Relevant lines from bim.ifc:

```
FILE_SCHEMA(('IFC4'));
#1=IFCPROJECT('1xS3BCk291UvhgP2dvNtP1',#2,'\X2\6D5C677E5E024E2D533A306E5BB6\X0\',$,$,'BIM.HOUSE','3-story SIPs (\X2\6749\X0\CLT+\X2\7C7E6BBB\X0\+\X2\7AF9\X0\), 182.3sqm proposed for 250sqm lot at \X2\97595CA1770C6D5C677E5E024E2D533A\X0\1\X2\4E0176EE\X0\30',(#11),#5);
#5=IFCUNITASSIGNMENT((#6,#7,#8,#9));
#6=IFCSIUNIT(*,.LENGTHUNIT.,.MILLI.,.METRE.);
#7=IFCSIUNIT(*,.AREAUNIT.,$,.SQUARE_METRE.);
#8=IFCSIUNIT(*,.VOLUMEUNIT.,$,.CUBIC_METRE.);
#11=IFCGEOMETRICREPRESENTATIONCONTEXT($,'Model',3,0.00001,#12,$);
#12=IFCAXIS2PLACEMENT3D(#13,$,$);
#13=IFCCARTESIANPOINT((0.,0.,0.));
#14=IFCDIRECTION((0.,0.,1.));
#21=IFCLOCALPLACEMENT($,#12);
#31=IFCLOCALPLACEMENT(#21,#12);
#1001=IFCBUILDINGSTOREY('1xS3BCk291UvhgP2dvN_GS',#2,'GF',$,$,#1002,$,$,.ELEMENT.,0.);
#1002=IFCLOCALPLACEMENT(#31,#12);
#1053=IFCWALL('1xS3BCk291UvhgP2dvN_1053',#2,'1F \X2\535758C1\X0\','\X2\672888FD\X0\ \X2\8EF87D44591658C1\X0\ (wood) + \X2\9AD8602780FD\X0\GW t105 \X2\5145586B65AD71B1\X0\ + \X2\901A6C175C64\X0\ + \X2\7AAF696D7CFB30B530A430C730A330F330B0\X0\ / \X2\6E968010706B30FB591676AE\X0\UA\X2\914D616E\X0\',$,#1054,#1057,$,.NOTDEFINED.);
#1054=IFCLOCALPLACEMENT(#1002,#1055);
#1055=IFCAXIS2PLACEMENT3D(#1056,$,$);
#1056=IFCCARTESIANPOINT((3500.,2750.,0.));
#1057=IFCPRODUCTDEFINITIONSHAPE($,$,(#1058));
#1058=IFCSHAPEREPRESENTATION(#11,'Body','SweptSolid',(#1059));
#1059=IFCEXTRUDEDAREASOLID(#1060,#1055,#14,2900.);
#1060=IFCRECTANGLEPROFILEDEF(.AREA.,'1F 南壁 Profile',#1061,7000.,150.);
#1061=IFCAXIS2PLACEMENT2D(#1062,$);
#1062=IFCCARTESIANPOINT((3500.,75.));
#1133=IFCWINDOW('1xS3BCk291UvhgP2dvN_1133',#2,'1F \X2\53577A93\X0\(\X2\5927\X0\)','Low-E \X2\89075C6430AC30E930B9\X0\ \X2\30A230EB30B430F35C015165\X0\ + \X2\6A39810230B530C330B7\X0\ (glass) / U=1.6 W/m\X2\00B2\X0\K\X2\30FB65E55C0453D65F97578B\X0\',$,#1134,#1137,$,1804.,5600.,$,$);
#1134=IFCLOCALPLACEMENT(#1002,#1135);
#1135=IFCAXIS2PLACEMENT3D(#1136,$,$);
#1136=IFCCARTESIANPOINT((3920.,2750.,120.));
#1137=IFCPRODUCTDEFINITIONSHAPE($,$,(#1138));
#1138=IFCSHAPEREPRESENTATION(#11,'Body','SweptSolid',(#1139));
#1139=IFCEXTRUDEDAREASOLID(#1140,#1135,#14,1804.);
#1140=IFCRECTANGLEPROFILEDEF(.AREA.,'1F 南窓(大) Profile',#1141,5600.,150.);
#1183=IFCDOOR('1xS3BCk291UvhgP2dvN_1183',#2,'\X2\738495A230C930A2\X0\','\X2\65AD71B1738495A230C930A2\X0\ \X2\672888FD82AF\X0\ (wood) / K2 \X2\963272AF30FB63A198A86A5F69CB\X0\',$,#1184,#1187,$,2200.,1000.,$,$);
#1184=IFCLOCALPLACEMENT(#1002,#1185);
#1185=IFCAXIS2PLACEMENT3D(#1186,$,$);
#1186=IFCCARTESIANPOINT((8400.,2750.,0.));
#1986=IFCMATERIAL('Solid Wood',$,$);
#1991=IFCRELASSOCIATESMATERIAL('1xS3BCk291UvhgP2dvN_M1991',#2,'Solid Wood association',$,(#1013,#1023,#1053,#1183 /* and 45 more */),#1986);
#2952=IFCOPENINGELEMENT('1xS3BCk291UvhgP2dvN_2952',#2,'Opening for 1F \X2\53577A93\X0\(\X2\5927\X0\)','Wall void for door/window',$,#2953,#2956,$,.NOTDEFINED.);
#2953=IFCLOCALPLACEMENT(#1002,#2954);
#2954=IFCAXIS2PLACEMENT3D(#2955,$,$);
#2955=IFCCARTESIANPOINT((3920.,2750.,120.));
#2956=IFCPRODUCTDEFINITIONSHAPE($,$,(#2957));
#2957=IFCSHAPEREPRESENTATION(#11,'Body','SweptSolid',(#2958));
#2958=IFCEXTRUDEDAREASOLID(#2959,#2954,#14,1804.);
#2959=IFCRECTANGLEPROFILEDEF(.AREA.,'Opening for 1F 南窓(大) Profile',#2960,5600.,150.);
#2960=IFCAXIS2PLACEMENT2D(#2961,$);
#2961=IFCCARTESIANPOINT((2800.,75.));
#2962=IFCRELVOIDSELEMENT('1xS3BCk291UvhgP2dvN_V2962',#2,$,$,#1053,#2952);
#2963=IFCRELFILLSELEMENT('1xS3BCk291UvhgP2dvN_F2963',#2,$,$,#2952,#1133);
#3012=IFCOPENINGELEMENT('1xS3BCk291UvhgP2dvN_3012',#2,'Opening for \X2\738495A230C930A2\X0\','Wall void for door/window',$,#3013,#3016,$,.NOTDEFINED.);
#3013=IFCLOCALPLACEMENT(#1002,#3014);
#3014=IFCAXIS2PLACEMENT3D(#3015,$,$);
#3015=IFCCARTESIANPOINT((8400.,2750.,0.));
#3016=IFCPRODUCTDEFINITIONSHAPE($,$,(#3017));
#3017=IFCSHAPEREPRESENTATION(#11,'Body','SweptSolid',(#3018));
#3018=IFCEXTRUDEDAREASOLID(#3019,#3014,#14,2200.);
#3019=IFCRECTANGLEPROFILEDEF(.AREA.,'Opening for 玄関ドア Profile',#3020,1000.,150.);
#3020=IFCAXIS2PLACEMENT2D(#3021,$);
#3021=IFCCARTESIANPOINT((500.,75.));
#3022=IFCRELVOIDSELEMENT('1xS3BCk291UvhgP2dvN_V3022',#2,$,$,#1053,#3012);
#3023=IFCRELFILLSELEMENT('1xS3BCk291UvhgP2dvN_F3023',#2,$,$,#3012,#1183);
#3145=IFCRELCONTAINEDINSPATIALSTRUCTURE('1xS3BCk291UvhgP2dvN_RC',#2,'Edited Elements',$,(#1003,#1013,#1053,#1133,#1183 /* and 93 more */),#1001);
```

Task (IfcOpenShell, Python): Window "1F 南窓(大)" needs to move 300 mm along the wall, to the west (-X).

```python
import ifcopenshell
import ifcopenshell.api.geometry
import ifcopenshell.util.placement
import ifcopenshell.util.unit

model = ifcopenshell.open("bim.ifc")
unit_scale = ifcopenshell.util.unit.calculate_unit_scale(model)

window = model.by_id(1133)
opening = window.FillsVoids[0].RelatingOpeningElement
wall = opening.VoidsElements[0].RelatingBuildingElement

wall_matrix = ifcopenshell.util.placement.get_local_placement(wall.ObjectPlacement)
shift = wall_matrix[:3, 0] * -0.3 / unit_scale
before = ifcopenshell.util.placement.get_local_placement(window.ObjectPlacement)[:3, 3].copy()

# The window is not placed relative to its opening, so move both.
for product in (opening, window):
    matrix = ifcopenshell.util.placement.get_local_placement(product.ObjectPlacement)
    matrix[:3, 3] += shift
    ifcopenshell.api.geometry.edit_object_placement(model, product=product, matrix=matrix, is_si=False)

after = ifcopenshell.util.placement.get_local_placement(window.ObjectPlacement)[:3, 3]
print("window moved by", (after - before).round(3) + 0.0)

model.write("bim_rev.ifc")
```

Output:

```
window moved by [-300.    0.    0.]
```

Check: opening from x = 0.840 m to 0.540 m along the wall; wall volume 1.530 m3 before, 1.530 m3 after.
